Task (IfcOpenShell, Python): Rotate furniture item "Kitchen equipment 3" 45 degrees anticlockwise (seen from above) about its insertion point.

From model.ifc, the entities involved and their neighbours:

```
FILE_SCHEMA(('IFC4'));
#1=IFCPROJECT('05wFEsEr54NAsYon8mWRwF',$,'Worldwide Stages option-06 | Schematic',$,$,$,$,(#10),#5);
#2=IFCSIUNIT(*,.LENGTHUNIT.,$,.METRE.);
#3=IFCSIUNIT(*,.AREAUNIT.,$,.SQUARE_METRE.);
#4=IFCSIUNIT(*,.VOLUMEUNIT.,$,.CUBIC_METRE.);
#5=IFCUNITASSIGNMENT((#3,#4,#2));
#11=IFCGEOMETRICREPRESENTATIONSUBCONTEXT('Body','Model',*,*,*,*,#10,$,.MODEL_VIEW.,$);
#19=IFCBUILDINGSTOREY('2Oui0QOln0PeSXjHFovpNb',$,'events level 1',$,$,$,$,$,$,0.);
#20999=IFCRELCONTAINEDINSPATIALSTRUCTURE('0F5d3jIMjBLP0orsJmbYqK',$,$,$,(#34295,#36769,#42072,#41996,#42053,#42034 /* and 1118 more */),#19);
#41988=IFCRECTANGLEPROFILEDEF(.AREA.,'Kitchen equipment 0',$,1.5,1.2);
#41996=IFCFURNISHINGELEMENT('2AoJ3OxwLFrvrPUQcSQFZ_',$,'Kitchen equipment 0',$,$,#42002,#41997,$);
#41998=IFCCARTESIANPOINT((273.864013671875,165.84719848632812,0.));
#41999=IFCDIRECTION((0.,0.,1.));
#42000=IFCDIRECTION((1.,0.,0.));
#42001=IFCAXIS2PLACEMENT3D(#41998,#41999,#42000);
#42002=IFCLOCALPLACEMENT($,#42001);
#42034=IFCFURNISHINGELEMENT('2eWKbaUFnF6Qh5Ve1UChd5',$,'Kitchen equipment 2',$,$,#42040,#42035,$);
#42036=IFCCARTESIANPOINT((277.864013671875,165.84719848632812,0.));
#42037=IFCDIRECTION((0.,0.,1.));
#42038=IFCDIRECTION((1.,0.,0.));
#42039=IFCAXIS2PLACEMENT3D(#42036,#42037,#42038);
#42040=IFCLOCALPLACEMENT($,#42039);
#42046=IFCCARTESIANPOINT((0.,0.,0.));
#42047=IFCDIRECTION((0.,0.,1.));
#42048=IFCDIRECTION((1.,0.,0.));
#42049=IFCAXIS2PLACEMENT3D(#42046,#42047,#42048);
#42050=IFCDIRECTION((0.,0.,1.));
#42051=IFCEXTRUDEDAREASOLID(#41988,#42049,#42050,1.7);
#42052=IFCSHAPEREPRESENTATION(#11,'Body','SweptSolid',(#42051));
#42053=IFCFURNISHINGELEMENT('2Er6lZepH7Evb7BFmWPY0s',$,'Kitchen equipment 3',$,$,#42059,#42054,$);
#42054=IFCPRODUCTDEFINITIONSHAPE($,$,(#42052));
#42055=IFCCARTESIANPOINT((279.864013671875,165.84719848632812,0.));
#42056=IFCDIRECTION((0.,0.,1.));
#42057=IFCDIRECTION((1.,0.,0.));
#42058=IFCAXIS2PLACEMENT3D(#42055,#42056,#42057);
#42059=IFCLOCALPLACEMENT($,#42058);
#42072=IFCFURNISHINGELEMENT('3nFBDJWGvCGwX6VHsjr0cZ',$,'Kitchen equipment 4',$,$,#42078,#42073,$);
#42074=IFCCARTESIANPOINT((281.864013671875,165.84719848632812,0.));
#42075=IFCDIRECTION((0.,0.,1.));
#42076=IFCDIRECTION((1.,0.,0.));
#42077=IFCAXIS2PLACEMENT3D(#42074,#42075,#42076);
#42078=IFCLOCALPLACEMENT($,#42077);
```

```python
import ifcopenshell
import ifcopenshell.api.geometry
import ifcopenshell.util.placement

model = ifcopenshell.open("model.ifc")

item = model.by_id(42053)
matrix = ifcopenshell.util.placement.get_local_placement(item.ObjectPlacement)
matrix = matrix @ ifcopenshell.util.placement.rotation(45, "Z")
ifcopenshell.api.geometry.edit_object_placement(model, product=item, matrix=matrix, is_si=False)

print(ifcopenshell.util.placement.get_local_placement(item.ObjectPlacement).round(3) + 0.0)

model.write("model_v2.ifc")
```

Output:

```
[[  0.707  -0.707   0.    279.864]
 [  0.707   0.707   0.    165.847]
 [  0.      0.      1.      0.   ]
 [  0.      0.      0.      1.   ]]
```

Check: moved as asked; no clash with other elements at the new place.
